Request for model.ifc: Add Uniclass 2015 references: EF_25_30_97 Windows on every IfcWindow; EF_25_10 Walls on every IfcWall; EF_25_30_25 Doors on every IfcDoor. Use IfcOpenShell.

First a look at what the model holds.

```python
import ifcopenshell

model = ifcopenshell.open("model.ifc")
print(model.schema)
print("classifications:", [c.Name for c in model.by_type("IfcClassification")])
for ifc_class in ("IfcDoor", "IfcRoof", "IfcStair", "IfcWall", "IfcWindow"):
    print(ifc_class, len(model.by_type(ifc_class)))
```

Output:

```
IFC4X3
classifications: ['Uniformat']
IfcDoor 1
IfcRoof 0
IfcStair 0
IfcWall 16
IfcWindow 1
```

```python
import ifcopenshell
import ifcopenshell.api.classification

model = ifcopenshell.open("model.ifc")

system = ifcopenshell.api.classification.add_classification(model, classification="Uniclass 2015")

codes = {
    "IfcWindow": ("EF_25_30_97", "Windows"),
    "IfcWall": ("EF_25_10", "Walls"),
    "IfcDoor": ("EF_25_30_25", "Doors"),
}
for ifc_class, (code, name) in codes.items():
    products = model.by_type(ifc_class)
    ifcopenshell.api.classification.add_reference(
        model, products=products, classification=system, identification=code, name=name
    )
    print(code, len(products))

model.write("model-out.ifc")
```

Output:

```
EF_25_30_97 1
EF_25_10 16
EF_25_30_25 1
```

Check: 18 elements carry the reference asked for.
